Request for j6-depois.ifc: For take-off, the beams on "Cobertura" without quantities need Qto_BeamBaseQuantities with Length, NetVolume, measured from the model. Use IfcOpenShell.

First a look at what the model holds.

```python
import ifcopenshell
import ifcopenshell.util.element
import ifcopenshell.util.unit

model = ifcopenshell.open("j6-depois.ifc")
print(model.schema)
for unit_type in ("LENGTHUNIT", "AREAUNIT", "VOLUMEUNIT"):
    print(unit_type, ifcopenshell.util.unit.calculate_unit_scale(model, unit_type))
storey = next(s for s in model.by_type("IfcBuildingStorey") if s.Name == "Cobertura")
beams = [e for e in ifcopenshell.util.element.get_decomposition(storey) if e.is_a("IfcBeam")]
for e in sorted(beams, key=lambda e: e.id()):
    print(e.id(), e.is_a(), e.Name, list(ifcopenshell.util.element.get_psets(e, qtos_only=True)), sep=" | ")
```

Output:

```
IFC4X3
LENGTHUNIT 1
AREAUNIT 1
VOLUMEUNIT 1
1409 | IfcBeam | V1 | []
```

```python
import ifcopenshell
import ifcopenshell.api.pset
import ifcopenshell.geom
import ifcopenshell.util.element
import ifcopenshell.util.shape
import ifcopenshell.util.unit

model = ifcopenshell.open("j6-depois.ifc")
unit_scale = ifcopenshell.util.unit.calculate_unit_scale(model)
volume_scale = ifcopenshell.util.unit.calculate_unit_scale(model, "VOLUMEUNIT")
settings = ifcopenshell.geom.settings()

storey = next(s for s in model.by_type("IfcBuildingStorey") if s.Name == "Cobertura")
beams = [e for e in ifcopenshell.util.element.get_decomposition(storey) if e.is_a("IfcBeam")]

for e in sorted(beams, key=lambda e: e.id()):
    if ifcopenshell.util.element.get_psets(e, qtos_only=True, should_inherit=False):
        continue
    # Geometry comes back in metres, in the element's own axes.
    shape = ifcopenshell.geom.create_shape(settings, e)
    values = {
        "Length": ifcopenshell.util.shape.get_max_xyz(shape.geometry) / unit_scale,
        "NetVolume": ifcopenshell.util.shape.get_volume(shape.geometry) / volume_scale,
    }
    qto = ifcopenshell.api.pset.add_qto(model, product=e, name="Qto_BeamBaseQuantities")
    ifcopenshell.api.pset.edit_qto(model, qto=qto, properties=values)
    print(e.id(), {k: round(v, 3) for k, v in values.items()})

model.write("j6-depois_updated.ifc")
```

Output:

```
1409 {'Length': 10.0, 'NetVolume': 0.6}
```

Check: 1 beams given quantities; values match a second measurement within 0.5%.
